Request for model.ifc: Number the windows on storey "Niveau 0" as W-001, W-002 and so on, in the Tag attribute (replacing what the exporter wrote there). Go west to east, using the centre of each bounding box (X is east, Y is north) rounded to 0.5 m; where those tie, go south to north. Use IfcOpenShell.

First a look at what the model holds.

```python
import ifcopenshell
import ifcopenshell.util.element
import ifcopenshell.util.placement

model = ifcopenshell.open("model.ifc")
print(model.schema)
storey = next(s for s in model.by_type("IfcBuildingStorey") if s.Name == "Niveau 0")
windows = [e for e in ifcopenshell.util.element.get_decomposition(storey) if e.is_a("IfcWindow")]
for e in sorted(windows, key=lambda e: e.id()):
    origin = ifcopenshell.util.placement.get_local_placement(e.ObjectPlacement)[:3, 3]
    print(e.id(), e.Tag, e.Name, origin.round(2) + 0.0, sep=" | ")
```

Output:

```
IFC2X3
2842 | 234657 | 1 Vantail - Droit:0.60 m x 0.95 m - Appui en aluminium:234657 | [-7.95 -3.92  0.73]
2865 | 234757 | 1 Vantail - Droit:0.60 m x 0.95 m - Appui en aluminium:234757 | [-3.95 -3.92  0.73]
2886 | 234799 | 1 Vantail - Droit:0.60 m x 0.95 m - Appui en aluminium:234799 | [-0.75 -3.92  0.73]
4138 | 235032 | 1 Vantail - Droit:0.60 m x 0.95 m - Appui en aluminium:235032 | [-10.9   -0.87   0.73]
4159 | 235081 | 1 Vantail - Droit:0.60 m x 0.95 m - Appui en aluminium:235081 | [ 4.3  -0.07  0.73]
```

```python
import ifcopenshell
import ifcopenshell.geom
import ifcopenshell.util.element
import ifcopenshell.util.shape

model = ifcopenshell.open("model.ifc")
settings = ifcopenshell.geom.settings()
settings.set("use-world-coords", True)


def centre(element):
    shape = ifcopenshell.geom.create_shape(settings, element)
    return ifcopenshell.util.shape.get_bbox_centroid(shape.geometry)


storey = next(s for s in model.by_type("IfcBuildingStorey") if s.Name == "Niveau 0")
windows = [e for e in ifcopenshell.util.element.get_decomposition(storey) if e.is_a("IfcWindow")]

# Insertion points can sit at a corner or the storey origin, so sort by the geometry (in metres).
centres = {e: centre(e) for e in windows}
windows.sort(key=lambda e: (round(centres[e][0] / 0.5), centres[e][1]))

for i, e in enumerate(windows, start=1):
    number = f"W-0{i:02d}"
    e.Tag = number
    print(e.id(), number)

model.write("model_updated.ifc")
```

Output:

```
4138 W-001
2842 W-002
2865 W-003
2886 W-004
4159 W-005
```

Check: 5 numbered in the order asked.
